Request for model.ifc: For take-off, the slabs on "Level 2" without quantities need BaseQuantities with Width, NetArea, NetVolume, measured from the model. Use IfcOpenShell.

First a look at what the model holds.

```python
import ifcopenshell
import ifcopenshell.util.element
import ifcopenshell.util.unit

model = ifcopenshell.open("model.ifc")
print(model.schema)
for unit_type in ("LENGTHUNIT", "AREAUNIT", "VOLUMEUNIT"):
    print(unit_type, ifcopenshell.util.unit.calculate_unit_scale(model, unit_type))
storey = next(s for s in model.by_type("IfcBuildingStorey") if s.Name == "Level 2")
slabs = [e for e in ifcopenshell.util.element.get_decomposition(storey) if e.is_a("IfcSlab")]
for e in sorted(slabs, key=lambda e: e.id()):
    print(e.id(), e.is_a(), e.Name, list(ifcopenshell.util.element.get_psets(e, qtos_only=True)), sep=" | ")
```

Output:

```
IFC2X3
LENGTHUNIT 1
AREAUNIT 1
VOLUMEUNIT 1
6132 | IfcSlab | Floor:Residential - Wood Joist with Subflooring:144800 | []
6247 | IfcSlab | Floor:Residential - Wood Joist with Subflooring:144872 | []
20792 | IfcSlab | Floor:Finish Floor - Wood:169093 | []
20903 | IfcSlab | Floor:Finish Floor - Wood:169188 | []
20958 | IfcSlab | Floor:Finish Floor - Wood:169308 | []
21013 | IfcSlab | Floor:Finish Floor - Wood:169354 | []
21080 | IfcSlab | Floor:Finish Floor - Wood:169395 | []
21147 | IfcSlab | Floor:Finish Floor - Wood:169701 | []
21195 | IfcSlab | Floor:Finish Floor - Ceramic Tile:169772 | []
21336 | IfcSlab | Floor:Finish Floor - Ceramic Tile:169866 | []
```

```python
import ifcopenshell
import ifcopenshell.api.pset
import ifcopenshell.geom
import ifcopenshell.util.element
import ifcopenshell.util.shape
import ifcopenshell.util.unit

model = ifcopenshell.open("model.ifc")
unit_scale = ifcopenshell.util.unit.calculate_unit_scale(model)
area_scale = ifcopenshell.util.unit.calculate_unit_scale(model, "AREAUNIT")
volume_scale = ifcopenshell.util.unit.calculate_unit_scale(model, "VOLUMEUNIT")
settings = ifcopenshell.geom.settings()

storey = next(s for s in model.by_type("IfcBuildingStorey") if s.Name == "Level 2")
slabs = [e for e in ifcopenshell.util.element.get_decomposition(storey) if e.is_a("IfcSlab")]

for e in sorted(slabs, key=lambda e: e.id()):
    if ifcopenshell.util.element.get_psets(e, qtos_only=True, should_inherit=False):
        continue
    # Geometry comes back in metres, in the element's own axes.
    shape = ifcopenshell.geom.create_shape(settings, e)
    values = {
        "Width": ifcopenshell.util.shape.get_z(shape.geometry) / unit_scale,
        "NetArea": ifcopenshell.util.shape.get_footprint_area(shape.geometry) / area_scale,
        "NetVolume": ifcopenshell.util.shape.get_volume(shape.geometry) / volume_scale,
    }
    qto = ifcopenshell.api.pset.add_qto(model, product=e, name="BaseQuantities")
    ifcopenshell.api.pset.edit_qto(model, qto=qto, properties=values)
    print(e.id(), {k: round(v, 3) for k, v in values.items()})

model.write("model_rev.ifc")
```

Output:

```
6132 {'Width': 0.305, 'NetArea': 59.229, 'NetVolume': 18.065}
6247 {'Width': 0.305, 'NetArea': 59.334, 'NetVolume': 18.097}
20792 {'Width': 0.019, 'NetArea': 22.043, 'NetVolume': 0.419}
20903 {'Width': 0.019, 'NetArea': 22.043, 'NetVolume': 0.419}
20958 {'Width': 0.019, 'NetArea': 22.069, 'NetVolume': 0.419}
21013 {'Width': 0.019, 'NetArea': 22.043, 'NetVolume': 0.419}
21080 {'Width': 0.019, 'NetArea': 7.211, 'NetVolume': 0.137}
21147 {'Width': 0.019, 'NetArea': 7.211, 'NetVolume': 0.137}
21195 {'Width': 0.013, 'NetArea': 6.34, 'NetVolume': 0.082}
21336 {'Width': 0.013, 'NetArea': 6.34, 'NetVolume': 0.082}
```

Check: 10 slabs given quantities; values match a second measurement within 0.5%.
